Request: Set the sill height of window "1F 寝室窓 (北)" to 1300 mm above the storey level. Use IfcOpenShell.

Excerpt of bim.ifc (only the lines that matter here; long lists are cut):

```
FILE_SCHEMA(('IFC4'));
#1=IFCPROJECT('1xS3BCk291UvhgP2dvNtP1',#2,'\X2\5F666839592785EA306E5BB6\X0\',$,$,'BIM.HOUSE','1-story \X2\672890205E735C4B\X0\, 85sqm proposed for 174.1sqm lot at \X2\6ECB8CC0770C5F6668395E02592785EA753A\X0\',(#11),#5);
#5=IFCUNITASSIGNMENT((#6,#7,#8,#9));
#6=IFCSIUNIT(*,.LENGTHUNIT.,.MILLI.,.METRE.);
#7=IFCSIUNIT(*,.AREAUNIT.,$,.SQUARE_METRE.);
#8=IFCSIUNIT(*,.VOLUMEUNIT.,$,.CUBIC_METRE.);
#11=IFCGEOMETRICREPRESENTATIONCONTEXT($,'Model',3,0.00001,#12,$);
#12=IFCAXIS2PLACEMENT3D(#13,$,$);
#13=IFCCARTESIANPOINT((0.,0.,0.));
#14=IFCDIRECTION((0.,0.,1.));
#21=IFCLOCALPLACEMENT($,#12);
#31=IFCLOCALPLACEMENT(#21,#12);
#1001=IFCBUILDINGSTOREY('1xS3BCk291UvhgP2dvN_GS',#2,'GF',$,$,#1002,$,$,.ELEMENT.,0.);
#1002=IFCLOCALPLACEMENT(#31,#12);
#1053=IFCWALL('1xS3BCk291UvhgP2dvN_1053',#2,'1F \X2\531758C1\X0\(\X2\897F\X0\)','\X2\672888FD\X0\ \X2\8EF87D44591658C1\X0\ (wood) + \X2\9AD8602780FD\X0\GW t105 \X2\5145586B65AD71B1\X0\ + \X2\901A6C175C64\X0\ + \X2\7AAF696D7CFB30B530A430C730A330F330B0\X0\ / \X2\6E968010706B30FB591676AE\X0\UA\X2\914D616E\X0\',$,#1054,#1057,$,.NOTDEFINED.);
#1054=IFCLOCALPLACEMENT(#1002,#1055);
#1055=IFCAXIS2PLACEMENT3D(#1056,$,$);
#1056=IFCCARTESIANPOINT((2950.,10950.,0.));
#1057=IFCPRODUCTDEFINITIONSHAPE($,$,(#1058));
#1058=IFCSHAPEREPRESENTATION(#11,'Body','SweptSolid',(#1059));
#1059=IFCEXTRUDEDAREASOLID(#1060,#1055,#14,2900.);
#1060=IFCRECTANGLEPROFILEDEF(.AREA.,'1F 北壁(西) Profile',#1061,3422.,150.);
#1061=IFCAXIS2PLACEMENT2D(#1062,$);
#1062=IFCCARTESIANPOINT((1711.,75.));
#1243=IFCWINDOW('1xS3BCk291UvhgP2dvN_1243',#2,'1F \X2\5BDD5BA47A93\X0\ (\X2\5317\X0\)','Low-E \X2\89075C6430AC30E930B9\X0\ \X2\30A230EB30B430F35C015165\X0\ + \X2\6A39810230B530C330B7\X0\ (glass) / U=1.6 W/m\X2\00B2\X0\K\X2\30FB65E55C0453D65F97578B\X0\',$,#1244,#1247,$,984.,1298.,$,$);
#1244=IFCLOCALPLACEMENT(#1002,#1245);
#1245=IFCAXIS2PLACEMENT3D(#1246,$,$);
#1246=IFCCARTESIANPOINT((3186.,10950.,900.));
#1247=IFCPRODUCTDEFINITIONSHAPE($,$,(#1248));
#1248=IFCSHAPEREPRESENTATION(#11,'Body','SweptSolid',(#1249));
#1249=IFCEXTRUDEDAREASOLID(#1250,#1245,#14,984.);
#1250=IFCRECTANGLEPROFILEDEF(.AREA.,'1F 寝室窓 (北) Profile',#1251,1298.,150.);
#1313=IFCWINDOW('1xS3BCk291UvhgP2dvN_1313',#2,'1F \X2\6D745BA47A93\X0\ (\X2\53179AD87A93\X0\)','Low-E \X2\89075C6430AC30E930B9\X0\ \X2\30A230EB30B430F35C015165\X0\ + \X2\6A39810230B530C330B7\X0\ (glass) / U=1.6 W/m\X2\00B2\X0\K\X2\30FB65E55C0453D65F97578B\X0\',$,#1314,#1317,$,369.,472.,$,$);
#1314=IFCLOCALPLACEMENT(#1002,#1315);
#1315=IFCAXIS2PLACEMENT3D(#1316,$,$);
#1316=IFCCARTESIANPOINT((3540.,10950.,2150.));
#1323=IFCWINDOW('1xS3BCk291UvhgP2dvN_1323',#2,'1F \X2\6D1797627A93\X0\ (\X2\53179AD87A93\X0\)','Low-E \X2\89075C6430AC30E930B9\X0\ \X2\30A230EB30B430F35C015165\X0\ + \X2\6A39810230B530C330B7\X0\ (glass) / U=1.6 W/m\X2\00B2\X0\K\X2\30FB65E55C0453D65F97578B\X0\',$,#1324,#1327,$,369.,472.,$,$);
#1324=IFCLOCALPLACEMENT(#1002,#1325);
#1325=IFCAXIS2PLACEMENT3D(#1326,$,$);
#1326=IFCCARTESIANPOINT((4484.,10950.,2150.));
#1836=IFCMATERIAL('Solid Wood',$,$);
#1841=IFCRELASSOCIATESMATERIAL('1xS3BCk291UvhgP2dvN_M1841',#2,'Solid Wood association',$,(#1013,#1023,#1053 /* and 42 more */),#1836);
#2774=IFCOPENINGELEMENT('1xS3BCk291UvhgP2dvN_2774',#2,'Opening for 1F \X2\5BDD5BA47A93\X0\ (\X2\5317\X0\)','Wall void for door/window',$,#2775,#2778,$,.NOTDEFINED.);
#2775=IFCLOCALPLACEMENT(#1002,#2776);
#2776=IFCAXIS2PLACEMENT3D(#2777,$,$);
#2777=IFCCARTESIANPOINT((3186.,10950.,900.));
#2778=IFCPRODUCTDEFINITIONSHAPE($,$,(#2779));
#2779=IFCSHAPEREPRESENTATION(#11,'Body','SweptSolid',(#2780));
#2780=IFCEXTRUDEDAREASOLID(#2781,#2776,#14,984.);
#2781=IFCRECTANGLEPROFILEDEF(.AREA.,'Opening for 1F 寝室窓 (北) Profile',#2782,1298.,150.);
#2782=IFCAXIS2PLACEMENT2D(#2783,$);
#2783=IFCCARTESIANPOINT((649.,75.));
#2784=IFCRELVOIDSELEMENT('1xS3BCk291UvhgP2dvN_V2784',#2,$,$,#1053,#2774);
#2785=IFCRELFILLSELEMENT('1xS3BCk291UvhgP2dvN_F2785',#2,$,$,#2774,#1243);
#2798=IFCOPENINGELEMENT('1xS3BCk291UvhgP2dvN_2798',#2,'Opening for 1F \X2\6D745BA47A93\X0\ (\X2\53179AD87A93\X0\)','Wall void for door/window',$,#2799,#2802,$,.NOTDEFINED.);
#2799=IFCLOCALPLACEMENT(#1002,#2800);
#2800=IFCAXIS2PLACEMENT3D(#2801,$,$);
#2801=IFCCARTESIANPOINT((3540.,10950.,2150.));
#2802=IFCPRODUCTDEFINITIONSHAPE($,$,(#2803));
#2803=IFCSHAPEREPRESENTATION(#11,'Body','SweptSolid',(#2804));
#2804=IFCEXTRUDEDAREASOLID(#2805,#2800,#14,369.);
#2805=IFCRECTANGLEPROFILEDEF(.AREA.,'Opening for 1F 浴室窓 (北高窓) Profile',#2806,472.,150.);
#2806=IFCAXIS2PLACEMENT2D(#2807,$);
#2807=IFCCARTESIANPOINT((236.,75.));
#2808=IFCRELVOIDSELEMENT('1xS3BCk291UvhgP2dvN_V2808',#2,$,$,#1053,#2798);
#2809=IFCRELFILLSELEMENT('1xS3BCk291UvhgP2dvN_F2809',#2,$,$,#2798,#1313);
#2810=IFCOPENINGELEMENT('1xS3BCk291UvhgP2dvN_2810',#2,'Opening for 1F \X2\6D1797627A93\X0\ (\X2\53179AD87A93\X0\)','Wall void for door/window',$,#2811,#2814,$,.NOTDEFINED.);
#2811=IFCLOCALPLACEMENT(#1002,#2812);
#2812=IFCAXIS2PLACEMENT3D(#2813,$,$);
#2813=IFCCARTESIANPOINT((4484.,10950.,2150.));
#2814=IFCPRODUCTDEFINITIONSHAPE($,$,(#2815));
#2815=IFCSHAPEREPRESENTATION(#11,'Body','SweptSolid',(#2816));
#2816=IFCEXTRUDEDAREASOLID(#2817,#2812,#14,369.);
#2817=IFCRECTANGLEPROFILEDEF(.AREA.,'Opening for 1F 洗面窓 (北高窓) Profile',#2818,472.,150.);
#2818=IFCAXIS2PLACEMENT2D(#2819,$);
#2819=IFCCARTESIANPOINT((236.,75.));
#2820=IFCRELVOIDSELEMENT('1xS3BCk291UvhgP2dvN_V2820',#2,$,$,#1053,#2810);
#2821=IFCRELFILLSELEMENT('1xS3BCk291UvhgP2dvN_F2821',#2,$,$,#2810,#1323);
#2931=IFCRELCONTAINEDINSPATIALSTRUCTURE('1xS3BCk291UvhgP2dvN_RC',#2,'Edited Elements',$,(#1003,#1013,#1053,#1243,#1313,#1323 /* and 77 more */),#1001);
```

```python
import numpy as np
import ifcopenshell
import ifcopenshell.api.geometry
import ifcopenshell.geom
import ifcopenshell.util.element
import ifcopenshell.util.placement
import ifcopenshell.util.shape
import ifcopenshell.util.unit

model = ifcopenshell.open("bim.ifc")
unit_scale = ifcopenshell.util.unit.calculate_unit_scale(model)

window = model.by_guid("1xS3BCk291UvhgP2dvN_1243")
opening = window.FillsVoids[0].RelatingOpeningElement
storey = ifcopenshell.util.element.get_container(window, ifc_class="IfcBuildingStorey")
level = ifcopenshell.util.placement.get_local_placement(storey.ObjectPlacement)[2, 3]

# The opening's origin need not be at the sill, so measure its lowest point.
shape = ifcopenshell.geom.create_shape(ifcopenshell.geom.settings(), opening)
bottom = ifcopenshell.util.shape.get_shape_bottom_elevation(shape, shape.geometry) / unit_scale
dz = level + 1.3 / unit_scale - bottom

shift = np.array([0.0, 0.0, dz])
# The window is not placed relative to its opening, so move both.
for product in (opening, window):
    matrix = ifcopenshell.util.placement.get_local_placement(product.ObjectPlacement)
    matrix[:3, 3] += shift
    ifcopenshell.api.geometry.edit_object_placement(model, product=product, matrix=matrix, is_si=False)

print(f"moved by {dz * unit_scale:+.3f} m")

model.write("bim_updated.ifc")
```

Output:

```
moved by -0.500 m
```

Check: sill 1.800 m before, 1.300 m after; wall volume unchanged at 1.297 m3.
